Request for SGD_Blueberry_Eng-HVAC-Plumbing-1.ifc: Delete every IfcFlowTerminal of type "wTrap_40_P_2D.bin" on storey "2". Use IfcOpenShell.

First a look at what the model holds.

```python
import ifcopenshell
import ifcopenshell.util.element

model = ifcopenshell.open("SGD_Blueberry_Eng-HVAC-Plumbing-1.ifc")
print(model.schema)
storey = next(s for s in model.by_type("IfcBuildingStorey") if s.Name == "2")
terminals = [e for e in ifcopenshell.util.element.get_decomposition(storey) if e.is_a("IfcFlowTerminal")]
seen = {}
for e in terminals:
    element_type = ifcopenshell.util.element.get_type(e)
    name = element_type.Name if element_type not in (None, e) else None
    seen[name] = seen.get(name, 0) + 1
for name, count in sorted(seen.items(), key=str):
    print(count, "x", name)
```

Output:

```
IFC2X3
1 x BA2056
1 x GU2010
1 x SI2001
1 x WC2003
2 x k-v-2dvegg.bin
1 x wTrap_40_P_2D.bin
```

```python
import ifcopenshell
import ifcopenshell.api.root
import ifcopenshell.util.element

model = ifcopenshell.open("SGD_Blueberry_Eng-HVAC-Plumbing-1.ifc")

storey = next(s for s in model.by_type("IfcBuildingStorey") if s.Name == "2")
terminals = [e for e in ifcopenshell.util.element.get_decomposition(storey) if e.is_a("IfcFlowTerminal")]
targets = [e for e in terminals if (t := ifcopenshell.util.element.get_type(e)) not in (None, e) and t.Name == "wTrap_40_P_2D.bin"]

for e in targets:
    ifcopenshell.api.root.remove_product(model, product=e)
print(len(targets), "removed")

model.write("SGD_Blueberry_Eng-HVAC-Plumbing-1_rev.ifc")
```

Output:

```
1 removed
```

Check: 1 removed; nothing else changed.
